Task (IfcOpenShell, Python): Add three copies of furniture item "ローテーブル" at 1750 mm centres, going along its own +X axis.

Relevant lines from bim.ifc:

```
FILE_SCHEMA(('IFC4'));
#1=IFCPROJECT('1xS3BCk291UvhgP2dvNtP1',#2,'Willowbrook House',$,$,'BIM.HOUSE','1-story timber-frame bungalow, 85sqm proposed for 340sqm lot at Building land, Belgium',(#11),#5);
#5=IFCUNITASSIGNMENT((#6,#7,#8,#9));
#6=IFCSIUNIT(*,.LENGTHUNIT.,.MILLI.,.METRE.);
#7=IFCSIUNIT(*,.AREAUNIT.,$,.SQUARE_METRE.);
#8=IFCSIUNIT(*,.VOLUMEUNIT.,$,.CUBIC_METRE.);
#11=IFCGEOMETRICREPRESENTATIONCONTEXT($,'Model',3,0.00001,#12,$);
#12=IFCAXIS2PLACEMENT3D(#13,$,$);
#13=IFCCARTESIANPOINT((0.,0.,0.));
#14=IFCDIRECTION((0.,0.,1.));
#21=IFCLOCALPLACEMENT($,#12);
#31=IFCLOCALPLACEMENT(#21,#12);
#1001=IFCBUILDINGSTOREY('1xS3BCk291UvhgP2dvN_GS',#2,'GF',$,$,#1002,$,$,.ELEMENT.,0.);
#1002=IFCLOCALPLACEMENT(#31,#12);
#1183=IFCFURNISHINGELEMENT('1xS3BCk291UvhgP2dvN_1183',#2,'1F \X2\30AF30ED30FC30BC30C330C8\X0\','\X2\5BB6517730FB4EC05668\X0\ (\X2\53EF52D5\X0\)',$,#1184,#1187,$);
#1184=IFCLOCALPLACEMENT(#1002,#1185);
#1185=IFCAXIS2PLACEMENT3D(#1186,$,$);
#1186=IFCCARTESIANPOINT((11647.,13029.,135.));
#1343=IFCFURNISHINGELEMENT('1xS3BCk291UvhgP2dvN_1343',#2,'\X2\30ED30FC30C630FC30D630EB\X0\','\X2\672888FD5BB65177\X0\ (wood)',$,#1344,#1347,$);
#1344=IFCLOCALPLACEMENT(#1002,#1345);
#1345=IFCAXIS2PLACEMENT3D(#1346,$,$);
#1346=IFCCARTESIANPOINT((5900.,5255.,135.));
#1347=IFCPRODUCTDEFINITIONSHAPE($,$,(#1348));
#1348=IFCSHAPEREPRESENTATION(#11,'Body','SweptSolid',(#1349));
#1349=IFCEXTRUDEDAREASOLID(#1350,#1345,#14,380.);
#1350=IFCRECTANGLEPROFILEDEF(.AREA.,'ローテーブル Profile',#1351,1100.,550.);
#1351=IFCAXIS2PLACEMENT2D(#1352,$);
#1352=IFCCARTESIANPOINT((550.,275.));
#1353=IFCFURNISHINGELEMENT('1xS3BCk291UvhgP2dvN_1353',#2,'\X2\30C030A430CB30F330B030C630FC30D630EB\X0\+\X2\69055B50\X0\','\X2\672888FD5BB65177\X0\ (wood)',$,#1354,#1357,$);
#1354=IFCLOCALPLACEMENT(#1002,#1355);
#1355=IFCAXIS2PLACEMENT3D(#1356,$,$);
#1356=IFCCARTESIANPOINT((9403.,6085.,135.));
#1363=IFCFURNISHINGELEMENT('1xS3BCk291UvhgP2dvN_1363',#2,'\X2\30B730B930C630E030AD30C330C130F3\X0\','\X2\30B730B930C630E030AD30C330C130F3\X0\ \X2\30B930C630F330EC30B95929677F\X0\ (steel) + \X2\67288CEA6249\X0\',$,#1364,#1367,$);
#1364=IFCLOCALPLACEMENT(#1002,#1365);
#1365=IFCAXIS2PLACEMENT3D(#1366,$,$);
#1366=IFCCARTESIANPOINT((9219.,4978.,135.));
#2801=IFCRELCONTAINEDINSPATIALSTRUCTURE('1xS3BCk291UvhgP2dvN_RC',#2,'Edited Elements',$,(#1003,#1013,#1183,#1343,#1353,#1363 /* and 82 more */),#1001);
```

```python
import ifcopenshell
import ifcopenshell.api.geometry
import ifcopenshell.api.root
import ifcopenshell.util.element
import ifcopenshell.util.placement
import ifcopenshell.util.unit

model = ifcopenshell.open("bim.ifc")
unit_scale = ifcopenshell.util.unit.calculate_unit_scale(model)


def reuse_history(source, copy):
    """copy_class also copies each property set's owner history, people and application; keep the originals."""
    for rel in copy.IsDefinedBy:
        if rel.is_a("IfcRelDefinesByProperties") and (history := rel.RelatingPropertyDefinition.OwnerHistory):
            rel.RelatingPropertyDefinition.OwnerHistory = source.OwnerHistory
            ifcopenshell.util.element.remove_deep2(model, history)


source = model.by_guid("1xS3BCk291UvhgP2dvN_1343")
base = ifcopenshell.util.placement.get_local_placement(source.ObjectPlacement)
step = base[:3, 0] * 1.75 / unit_scale

for i in range(1, 4):
    copy = ifcopenshell.api.root.copy_class(model, product=source)
    copy.Representation = ifcopenshell.util.element.copy_deep(
        model, source.Representation, exclude=["IfcGeometricRepresentationContext", "IfcRepresentationMap"]
    )
    reuse_history(source, copy)
    matrix = base.copy()
    matrix[:3, 3] += i * step
    print("added at", matrix[:3, 3].round(3) + 0.0)
    ifcopenshell.api.geometry.edit_object_placement(model, product=copy, matrix=matrix, is_si=False)

model.write("bim_rev.ifc")
```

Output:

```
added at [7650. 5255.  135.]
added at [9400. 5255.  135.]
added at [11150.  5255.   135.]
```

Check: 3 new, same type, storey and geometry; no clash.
